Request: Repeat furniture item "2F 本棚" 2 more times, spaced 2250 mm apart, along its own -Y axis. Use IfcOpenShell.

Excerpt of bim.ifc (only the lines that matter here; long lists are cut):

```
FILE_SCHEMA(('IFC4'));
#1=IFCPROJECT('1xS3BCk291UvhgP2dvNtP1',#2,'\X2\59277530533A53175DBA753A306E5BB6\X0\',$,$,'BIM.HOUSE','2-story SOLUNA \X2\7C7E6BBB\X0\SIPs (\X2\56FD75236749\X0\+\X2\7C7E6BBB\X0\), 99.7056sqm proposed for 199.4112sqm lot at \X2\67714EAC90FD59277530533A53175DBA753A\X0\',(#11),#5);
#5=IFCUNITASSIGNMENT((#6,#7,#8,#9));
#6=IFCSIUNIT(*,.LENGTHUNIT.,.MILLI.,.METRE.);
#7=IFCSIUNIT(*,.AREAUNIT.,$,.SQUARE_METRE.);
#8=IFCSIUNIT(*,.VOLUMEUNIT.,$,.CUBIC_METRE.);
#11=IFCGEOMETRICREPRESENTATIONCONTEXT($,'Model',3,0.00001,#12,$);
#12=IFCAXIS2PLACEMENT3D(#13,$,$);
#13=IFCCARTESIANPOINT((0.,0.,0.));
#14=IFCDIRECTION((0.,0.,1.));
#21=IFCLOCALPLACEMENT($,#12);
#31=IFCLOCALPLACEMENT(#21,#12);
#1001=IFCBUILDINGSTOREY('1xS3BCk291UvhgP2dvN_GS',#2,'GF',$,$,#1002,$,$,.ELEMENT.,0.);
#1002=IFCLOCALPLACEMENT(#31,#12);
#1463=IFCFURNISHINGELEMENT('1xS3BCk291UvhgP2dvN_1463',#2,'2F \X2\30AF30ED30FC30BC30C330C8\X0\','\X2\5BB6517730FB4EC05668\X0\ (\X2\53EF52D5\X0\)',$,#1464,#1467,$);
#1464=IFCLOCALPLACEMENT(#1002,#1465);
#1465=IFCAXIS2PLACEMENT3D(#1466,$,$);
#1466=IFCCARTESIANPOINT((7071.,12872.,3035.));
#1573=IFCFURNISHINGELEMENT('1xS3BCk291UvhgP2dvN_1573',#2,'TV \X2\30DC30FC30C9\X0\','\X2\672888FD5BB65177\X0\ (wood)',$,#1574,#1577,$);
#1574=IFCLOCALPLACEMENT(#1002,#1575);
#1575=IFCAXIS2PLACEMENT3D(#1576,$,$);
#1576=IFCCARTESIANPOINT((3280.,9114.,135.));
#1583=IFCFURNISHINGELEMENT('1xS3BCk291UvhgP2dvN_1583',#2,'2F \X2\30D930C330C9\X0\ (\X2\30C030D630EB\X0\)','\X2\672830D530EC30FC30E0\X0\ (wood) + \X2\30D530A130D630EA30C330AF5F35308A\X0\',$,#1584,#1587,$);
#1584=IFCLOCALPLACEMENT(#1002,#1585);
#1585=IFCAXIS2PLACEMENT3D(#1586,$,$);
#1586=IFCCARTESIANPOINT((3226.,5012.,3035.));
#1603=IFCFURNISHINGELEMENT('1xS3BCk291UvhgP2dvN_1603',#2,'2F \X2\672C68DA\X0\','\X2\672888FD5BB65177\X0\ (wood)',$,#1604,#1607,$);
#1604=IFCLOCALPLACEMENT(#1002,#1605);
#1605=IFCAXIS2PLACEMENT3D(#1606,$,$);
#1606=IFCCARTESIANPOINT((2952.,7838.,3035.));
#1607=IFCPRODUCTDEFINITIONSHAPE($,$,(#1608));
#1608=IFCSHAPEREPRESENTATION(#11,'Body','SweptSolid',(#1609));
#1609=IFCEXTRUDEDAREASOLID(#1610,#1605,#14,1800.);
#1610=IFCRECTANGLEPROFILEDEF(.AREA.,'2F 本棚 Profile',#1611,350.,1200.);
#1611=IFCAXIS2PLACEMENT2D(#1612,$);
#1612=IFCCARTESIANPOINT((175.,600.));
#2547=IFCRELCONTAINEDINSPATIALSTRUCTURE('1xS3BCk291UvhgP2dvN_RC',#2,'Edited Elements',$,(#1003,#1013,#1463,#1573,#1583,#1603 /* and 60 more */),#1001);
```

```python
import ifcopenshell
import ifcopenshell.api.geometry
import ifcopenshell.api.root
import ifcopenshell.util.element
import ifcopenshell.util.placement
import ifcopenshell.util.unit

model = ifcopenshell.open("bim.ifc")
unit_scale = ifcopenshell.util.unit.calculate_unit_scale(model)


def reuse_history(source, copy):
    """copy_class also copies each property set's owner history, people and application; keep the originals."""
    for rel in copy.IsDefinedBy:
        if rel.is_a("IfcRelDefinesByProperties") and (history := rel.RelatingPropertyDefinition.OwnerHistory):
            rel.RelatingPropertyDefinition.OwnerHistory = source.OwnerHistory
            ifcopenshell.util.element.remove_deep2(model, history)


source = model.by_guid("1xS3BCk291UvhgP2dvN_1603")
base = ifcopenshell.util.placement.get_local_placement(source.ObjectPlacement)
step = -base[:3, 1] * 2.25 / unit_scale

for i in range(1, 3):
    copy = ifcopenshell.api.root.copy_class(model, product=source)
    copy.Representation = ifcopenshell.util.element.copy_deep(
        model, source.Representation, exclude=["IfcGeometricRepresentationContext", "IfcRepresentationMap"]
    )
    reuse_history(source, copy)
    matrix = base.copy()
    matrix[:3, 3] += i * step
    print("added at", matrix[:3, 3].round(3) + 0.0)
    ifcopenshell.api.geometry.edit_object_placement(model, product=copy, matrix=matrix, is_si=False)

model.write("bim_rev.ifc")
```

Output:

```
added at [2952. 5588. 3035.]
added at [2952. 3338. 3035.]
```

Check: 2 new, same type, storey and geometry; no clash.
